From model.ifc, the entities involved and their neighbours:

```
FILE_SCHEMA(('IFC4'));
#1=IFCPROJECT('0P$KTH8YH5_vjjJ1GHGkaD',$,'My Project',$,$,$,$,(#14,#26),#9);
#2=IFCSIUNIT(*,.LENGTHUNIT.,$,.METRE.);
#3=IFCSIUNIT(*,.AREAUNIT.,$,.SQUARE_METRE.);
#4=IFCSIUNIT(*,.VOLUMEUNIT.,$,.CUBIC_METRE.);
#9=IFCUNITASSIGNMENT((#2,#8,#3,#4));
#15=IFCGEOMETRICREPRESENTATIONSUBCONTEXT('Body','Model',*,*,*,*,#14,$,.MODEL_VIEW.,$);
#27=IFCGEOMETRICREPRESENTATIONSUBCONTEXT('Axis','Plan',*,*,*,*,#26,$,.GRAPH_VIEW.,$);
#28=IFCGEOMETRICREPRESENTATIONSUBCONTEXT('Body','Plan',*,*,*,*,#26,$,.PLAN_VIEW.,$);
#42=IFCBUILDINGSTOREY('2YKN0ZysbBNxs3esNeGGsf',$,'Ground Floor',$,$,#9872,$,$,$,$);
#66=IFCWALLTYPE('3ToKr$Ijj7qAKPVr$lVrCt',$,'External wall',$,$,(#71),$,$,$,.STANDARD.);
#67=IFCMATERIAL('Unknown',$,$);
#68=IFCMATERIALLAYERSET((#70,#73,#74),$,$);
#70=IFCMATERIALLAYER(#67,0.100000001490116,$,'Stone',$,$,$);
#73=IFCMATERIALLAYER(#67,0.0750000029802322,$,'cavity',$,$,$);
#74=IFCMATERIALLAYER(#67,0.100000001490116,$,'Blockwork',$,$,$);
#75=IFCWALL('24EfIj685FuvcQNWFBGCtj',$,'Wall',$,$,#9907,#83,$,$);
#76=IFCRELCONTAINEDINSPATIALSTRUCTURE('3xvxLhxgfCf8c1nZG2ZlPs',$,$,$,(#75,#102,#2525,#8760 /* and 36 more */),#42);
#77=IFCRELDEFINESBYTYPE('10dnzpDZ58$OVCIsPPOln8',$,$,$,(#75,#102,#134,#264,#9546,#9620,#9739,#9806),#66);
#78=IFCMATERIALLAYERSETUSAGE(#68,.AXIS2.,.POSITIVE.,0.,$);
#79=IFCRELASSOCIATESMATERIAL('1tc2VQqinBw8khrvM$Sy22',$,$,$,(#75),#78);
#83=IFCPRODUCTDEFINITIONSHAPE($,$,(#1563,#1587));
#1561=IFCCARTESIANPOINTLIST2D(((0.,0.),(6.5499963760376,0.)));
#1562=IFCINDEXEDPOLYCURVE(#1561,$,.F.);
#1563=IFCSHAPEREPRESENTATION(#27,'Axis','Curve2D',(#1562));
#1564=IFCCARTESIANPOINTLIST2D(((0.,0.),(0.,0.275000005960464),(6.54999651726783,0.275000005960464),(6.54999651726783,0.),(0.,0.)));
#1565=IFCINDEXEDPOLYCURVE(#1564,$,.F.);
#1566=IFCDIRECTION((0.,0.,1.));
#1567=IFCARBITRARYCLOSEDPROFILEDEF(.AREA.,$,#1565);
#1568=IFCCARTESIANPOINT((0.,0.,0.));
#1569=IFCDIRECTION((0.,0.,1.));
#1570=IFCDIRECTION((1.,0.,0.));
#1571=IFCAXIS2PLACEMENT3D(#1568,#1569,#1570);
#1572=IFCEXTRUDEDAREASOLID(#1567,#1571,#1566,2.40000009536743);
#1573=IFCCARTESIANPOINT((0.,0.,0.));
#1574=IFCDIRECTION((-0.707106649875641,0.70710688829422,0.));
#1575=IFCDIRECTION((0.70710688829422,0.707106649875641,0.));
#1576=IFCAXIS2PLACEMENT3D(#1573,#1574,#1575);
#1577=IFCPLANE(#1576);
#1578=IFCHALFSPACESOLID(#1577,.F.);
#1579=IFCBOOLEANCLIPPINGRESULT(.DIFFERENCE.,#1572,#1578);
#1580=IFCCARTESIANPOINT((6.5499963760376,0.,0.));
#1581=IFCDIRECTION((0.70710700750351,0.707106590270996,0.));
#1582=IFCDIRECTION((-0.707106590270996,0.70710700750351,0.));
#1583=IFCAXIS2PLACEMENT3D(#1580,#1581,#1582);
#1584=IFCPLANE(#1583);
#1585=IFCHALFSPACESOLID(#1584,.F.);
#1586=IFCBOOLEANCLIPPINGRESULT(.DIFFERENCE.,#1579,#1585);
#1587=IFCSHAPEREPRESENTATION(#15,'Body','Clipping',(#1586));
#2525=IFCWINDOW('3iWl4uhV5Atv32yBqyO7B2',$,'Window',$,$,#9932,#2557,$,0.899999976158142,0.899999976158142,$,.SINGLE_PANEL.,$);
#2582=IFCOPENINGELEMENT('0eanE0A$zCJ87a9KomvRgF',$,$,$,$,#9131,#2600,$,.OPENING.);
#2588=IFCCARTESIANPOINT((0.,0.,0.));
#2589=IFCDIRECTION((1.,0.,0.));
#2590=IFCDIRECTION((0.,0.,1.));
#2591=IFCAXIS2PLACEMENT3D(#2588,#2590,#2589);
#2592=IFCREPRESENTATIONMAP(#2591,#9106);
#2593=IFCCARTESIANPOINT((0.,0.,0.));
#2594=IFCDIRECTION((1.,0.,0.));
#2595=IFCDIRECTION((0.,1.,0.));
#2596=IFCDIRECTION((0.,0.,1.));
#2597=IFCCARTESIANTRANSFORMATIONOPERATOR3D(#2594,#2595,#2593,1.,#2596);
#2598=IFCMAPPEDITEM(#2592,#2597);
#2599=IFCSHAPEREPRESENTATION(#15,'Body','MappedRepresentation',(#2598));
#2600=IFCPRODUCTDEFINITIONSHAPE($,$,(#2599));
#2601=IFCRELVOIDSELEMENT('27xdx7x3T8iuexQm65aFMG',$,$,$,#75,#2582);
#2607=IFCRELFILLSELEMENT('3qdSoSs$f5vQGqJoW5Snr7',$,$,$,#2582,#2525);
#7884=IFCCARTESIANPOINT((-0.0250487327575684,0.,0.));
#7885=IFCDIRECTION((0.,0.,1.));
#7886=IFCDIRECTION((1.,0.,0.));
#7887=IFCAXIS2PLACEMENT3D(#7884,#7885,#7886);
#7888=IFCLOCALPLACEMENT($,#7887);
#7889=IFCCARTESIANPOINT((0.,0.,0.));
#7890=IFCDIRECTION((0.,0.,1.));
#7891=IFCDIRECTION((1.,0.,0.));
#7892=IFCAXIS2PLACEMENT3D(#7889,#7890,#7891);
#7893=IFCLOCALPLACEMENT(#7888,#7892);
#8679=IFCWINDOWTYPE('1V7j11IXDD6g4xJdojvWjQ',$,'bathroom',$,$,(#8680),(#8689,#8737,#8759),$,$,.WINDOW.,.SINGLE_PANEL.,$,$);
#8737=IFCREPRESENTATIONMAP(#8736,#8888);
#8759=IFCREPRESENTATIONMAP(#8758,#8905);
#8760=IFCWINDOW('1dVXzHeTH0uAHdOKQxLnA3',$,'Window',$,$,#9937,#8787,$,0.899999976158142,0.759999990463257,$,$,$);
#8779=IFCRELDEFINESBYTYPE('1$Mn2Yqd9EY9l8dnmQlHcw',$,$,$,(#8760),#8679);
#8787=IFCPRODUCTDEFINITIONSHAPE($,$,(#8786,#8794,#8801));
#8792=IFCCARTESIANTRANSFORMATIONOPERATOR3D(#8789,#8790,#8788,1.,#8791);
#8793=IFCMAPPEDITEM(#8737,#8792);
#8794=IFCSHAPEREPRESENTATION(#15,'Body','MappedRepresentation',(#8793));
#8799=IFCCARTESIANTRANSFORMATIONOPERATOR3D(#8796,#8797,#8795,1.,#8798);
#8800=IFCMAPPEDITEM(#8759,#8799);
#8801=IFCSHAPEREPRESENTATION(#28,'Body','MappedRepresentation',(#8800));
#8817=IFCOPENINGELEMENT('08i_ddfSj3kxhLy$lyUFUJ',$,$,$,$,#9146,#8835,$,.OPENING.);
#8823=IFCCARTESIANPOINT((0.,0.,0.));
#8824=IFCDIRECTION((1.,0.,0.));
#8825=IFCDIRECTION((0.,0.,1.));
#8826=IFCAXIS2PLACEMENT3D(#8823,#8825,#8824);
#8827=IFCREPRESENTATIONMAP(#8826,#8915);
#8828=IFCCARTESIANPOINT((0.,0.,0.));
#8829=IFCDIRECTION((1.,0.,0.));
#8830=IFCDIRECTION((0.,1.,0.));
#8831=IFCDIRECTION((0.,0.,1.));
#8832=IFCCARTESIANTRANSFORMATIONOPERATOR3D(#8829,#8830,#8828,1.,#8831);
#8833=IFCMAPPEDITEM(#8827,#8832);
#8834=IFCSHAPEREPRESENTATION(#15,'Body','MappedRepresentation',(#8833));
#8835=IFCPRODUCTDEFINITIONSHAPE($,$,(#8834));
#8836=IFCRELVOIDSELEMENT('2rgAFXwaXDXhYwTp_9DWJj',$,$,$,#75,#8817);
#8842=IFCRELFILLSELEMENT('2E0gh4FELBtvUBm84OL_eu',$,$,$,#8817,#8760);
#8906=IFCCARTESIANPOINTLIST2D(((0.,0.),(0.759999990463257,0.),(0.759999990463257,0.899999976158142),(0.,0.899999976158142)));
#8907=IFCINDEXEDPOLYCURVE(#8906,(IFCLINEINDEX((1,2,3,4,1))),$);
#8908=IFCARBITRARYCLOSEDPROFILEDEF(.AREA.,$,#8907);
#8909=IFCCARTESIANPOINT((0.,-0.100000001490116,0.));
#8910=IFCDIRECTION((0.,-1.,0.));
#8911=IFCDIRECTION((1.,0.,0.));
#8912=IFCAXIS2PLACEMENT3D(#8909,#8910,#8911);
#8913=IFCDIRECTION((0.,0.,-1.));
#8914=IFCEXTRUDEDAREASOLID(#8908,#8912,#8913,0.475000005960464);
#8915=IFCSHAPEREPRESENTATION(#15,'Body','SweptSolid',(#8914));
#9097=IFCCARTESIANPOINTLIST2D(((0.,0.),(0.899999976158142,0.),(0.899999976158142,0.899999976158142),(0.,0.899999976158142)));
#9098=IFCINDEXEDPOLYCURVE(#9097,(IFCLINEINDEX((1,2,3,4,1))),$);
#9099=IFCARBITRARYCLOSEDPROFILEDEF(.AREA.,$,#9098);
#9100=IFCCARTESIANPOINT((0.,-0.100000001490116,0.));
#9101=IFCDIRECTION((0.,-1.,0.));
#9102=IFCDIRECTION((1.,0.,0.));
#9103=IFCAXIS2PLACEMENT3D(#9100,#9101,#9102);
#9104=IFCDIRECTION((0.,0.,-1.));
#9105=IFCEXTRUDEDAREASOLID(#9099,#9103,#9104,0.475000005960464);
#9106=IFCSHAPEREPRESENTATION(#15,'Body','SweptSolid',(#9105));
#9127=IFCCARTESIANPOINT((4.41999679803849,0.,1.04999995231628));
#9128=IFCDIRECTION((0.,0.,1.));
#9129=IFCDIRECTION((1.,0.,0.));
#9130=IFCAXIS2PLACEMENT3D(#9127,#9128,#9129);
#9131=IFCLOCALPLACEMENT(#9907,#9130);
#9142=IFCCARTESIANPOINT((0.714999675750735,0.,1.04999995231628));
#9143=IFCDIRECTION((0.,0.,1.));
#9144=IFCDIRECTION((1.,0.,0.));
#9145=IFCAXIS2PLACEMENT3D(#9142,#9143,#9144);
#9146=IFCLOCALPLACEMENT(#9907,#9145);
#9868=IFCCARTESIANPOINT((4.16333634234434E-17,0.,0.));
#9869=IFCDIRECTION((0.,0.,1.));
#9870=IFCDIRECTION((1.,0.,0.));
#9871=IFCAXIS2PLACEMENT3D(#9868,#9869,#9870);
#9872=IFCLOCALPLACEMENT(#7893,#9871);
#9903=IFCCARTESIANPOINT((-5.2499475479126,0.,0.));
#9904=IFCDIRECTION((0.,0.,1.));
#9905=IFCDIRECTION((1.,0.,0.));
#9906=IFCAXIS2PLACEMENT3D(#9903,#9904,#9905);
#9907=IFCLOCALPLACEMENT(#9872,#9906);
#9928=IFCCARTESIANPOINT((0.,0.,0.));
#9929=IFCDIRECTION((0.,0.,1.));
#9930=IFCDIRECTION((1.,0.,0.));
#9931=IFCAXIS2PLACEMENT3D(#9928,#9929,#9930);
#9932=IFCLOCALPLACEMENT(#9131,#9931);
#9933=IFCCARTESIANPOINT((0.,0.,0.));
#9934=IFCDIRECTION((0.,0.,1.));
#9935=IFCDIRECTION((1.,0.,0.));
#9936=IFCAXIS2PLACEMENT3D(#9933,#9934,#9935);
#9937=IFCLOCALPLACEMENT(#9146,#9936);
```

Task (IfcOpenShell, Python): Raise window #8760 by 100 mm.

```python
import numpy as np
import ifcopenshell
import ifcopenshell.api.geometry
import ifcopenshell.util.placement
import ifcopenshell.util.unit

model = ifcopenshell.open("model.ifc")
unit_scale = ifcopenshell.util.unit.calculate_unit_scale(model)

window = model.by_guid("1dVXzHeTH0uAHdOKQxLnA3")
opening = window.FillsVoids[0].RelatingOpeningElement
dz = 0.1 / unit_scale

shift = np.array([0.0, 0.0, dz])
# The window is placed relative to its opening, so it follows when the opening moves.
matrix = ifcopenshell.util.placement.get_local_placement(opening.ObjectPlacement)
matrix[:3, 3] += shift
ifcopenshell.api.geometry.edit_object_placement(
    model, product=opening, matrix=matrix, is_si=False, should_transform_children=True
)

print(f"moved by {dz * unit_scale:+.3f} m")

model.write("model-out.ifc")
```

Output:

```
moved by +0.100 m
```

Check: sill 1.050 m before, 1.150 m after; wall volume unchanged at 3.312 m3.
